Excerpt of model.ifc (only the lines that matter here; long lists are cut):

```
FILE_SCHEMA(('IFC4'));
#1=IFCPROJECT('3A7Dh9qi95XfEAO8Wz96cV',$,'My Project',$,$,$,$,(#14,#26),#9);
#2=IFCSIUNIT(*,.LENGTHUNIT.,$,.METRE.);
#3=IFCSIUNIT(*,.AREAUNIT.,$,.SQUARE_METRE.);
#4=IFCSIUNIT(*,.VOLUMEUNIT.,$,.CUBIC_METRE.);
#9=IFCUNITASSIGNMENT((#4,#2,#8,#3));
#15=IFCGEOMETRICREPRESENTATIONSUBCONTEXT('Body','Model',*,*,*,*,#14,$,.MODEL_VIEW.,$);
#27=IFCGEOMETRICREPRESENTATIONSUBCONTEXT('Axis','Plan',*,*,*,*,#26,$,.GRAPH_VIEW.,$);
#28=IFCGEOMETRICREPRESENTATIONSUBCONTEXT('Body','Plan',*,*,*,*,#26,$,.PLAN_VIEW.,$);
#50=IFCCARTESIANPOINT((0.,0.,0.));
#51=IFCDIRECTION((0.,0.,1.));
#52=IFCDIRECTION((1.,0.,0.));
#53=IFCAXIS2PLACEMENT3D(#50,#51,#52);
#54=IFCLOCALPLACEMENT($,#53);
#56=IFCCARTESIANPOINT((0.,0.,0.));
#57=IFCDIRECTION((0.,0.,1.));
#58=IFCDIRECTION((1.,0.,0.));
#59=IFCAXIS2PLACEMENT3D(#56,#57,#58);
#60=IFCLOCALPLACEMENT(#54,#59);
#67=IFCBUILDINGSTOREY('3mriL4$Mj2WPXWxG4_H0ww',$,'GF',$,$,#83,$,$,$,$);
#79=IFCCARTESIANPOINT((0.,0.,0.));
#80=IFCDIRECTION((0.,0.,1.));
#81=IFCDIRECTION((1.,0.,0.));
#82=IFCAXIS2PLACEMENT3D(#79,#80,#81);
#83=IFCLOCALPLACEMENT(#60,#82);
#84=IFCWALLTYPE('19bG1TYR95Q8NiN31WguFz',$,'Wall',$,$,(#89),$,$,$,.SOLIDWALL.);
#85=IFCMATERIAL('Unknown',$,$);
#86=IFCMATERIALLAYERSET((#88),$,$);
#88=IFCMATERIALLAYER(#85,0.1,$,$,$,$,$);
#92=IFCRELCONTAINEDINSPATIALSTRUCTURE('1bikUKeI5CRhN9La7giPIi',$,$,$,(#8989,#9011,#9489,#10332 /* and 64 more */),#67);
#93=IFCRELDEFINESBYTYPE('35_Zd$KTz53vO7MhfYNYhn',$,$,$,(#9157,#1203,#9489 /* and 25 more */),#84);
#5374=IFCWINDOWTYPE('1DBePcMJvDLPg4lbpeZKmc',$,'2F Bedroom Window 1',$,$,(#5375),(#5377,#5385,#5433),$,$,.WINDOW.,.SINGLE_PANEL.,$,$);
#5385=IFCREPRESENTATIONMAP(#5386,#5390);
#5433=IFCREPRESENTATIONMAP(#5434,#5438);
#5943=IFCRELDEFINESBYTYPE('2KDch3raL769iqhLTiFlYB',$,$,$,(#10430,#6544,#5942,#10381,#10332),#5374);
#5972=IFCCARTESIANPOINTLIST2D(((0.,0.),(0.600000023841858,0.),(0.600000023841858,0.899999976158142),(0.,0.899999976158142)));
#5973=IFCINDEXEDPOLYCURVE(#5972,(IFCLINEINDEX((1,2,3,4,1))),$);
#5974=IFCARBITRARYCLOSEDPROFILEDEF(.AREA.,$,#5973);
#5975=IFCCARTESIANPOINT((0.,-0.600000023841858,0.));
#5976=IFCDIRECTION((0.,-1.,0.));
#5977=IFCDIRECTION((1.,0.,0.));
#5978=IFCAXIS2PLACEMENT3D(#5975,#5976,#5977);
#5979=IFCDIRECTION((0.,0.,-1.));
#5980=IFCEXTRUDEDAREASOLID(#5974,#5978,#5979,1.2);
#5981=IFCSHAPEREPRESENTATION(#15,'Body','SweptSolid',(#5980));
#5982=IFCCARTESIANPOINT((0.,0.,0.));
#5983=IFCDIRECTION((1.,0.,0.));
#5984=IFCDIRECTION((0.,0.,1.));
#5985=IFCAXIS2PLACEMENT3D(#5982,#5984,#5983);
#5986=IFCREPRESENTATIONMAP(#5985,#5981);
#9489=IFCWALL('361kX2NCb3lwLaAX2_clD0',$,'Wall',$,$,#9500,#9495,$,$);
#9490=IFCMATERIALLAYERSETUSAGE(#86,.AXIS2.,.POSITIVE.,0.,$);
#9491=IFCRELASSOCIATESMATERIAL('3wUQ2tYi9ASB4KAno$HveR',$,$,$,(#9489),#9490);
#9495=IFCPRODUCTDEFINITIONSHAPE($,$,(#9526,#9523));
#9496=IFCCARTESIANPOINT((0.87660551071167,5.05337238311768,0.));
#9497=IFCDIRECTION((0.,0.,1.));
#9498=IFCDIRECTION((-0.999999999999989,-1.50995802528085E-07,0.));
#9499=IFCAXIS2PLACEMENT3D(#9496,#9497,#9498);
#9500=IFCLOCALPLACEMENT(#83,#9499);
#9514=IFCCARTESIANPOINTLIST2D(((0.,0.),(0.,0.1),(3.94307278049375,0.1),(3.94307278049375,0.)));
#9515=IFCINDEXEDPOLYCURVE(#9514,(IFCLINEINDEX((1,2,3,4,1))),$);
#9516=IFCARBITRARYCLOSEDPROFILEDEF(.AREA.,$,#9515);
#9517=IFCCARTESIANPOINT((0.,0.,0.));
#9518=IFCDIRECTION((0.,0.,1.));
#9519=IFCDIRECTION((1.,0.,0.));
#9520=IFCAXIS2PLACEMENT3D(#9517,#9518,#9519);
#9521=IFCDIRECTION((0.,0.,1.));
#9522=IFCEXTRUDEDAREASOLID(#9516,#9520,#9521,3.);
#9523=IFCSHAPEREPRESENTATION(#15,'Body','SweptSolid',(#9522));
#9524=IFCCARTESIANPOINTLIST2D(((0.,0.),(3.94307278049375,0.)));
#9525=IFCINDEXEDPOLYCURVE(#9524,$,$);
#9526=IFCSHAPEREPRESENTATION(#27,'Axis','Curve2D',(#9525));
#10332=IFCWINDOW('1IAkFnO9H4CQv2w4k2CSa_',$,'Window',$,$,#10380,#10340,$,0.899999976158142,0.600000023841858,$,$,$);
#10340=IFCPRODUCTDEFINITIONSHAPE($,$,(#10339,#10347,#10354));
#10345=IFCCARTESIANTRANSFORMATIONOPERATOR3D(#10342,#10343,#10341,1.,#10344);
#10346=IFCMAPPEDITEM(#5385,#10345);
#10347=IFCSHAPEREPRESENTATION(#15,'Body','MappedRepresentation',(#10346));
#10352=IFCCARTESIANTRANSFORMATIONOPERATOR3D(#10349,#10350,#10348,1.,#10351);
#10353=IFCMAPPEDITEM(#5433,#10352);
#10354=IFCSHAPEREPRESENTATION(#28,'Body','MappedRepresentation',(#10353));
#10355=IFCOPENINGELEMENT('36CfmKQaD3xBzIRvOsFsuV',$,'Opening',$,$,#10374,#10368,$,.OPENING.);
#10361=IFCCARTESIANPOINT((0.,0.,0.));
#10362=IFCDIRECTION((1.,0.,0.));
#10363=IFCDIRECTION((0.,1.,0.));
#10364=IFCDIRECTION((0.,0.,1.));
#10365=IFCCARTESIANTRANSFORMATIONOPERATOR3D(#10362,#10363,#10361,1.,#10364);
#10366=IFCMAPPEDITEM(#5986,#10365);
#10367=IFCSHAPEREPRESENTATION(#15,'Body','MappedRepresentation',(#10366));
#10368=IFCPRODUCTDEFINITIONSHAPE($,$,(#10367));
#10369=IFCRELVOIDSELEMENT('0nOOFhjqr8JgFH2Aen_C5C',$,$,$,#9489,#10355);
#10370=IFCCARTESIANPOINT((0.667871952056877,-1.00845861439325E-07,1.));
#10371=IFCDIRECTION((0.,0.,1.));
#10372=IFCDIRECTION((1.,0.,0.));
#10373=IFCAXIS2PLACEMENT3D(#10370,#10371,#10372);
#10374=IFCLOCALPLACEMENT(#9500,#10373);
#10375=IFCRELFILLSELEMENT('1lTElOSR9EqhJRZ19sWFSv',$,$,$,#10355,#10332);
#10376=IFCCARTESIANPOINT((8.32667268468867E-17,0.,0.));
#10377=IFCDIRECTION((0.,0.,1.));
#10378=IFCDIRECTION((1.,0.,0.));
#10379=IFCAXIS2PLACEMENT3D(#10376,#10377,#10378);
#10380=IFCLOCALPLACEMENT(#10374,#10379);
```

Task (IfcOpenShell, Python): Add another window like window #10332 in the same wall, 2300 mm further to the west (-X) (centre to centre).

```python
import ifcopenshell
import ifcopenshell.api.feature
import ifcopenshell.api.geometry
import ifcopenshell.api.root
import ifcopenshell.geom
import ifcopenshell.util.element
import ifcopenshell.util.placement
import ifcopenshell.util.shape

model = ifcopenshell.open("model.ifc")
settings = ifcopenshell.geom.settings()


def volume(element):
    """Net volume in cubic metres, openings subtracted."""
    shape = ifcopenshell.geom.create_shape(settings, element)
    return ifcopenshell.util.shape.get_volume(shape.geometry)


window = model.by_guid("1IAkFnO9H4CQv2w4k2CSa_")
opening = window.FillsVoids[0].RelatingOpeningElement
wall = opening.VoidsElements[0].RelatingBuildingElement
before = volume(wall)
shift = ifcopenshell.util.placement.get_local_placement(wall.ObjectPlacement)[:3, 0] * 2.3

# copy_class copies the void relationship, type, container and properties, but no geometry.
new_opening = ifcopenshell.api.root.copy_class(model, product=opening)
new_opening.Representation = ifcopenshell.util.element.copy_deep(
    model, opening.Representation, exclude=["IfcGeometricRepresentationContext", "IfcRepresentationMap"]
)
new_window = ifcopenshell.api.root.copy_class(model, product=window)
new_window.Representation = ifcopenshell.util.element.copy_deep(
    model, window.Representation, exclude=["IfcGeometricRepresentationContext", "IfcRepresentationMap"]
)
ifcopenshell.api.feature.add_filling(model, opening=new_opening, element=new_window)

for old, new in ((opening, new_opening), (window, new_window)):
    matrix = ifcopenshell.util.placement.get_local_placement(old.ObjectPlacement)
    matrix[:3, 3] += shift
    ifcopenshell.api.geometry.edit_object_placement(model, product=new, matrix=matrix, is_si=False)

after = volume(wall)

print(f"wall volume {before:.3f} -> {after:.3f} m3")

model.write("model-out.ifc")
```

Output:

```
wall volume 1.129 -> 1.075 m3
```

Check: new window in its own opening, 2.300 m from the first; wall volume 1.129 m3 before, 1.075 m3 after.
